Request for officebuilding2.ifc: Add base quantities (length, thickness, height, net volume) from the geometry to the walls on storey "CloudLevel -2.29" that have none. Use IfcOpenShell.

First a look at what the model holds.

```python
import ifcopenshell
import ifcopenshell.util.element
import ifcopenshell.util.unit

model = ifcopenshell.open("officebuilding2.ifc")
print(model.schema)
for unit_type in ("LENGTHUNIT", "AREAUNIT", "VOLUMEUNIT"):
    print(unit_type, ifcopenshell.util.unit.calculate_unit_scale(model, unit_type))
storey = next(s for s in model.by_type("IfcBuildingStorey") if s.Name == "CloudLevel -2.29")
walls = [e for e in ifcopenshell.util.element.get_decomposition(storey) if e.is_a("IfcWall")]
for e in sorted(walls, key=lambda e: e.id()):
    print(e.id(), e.is_a(), e.Name, list(ifcopenshell.util.element.get_psets(e, qtos_only=True)), sep=" | ")
```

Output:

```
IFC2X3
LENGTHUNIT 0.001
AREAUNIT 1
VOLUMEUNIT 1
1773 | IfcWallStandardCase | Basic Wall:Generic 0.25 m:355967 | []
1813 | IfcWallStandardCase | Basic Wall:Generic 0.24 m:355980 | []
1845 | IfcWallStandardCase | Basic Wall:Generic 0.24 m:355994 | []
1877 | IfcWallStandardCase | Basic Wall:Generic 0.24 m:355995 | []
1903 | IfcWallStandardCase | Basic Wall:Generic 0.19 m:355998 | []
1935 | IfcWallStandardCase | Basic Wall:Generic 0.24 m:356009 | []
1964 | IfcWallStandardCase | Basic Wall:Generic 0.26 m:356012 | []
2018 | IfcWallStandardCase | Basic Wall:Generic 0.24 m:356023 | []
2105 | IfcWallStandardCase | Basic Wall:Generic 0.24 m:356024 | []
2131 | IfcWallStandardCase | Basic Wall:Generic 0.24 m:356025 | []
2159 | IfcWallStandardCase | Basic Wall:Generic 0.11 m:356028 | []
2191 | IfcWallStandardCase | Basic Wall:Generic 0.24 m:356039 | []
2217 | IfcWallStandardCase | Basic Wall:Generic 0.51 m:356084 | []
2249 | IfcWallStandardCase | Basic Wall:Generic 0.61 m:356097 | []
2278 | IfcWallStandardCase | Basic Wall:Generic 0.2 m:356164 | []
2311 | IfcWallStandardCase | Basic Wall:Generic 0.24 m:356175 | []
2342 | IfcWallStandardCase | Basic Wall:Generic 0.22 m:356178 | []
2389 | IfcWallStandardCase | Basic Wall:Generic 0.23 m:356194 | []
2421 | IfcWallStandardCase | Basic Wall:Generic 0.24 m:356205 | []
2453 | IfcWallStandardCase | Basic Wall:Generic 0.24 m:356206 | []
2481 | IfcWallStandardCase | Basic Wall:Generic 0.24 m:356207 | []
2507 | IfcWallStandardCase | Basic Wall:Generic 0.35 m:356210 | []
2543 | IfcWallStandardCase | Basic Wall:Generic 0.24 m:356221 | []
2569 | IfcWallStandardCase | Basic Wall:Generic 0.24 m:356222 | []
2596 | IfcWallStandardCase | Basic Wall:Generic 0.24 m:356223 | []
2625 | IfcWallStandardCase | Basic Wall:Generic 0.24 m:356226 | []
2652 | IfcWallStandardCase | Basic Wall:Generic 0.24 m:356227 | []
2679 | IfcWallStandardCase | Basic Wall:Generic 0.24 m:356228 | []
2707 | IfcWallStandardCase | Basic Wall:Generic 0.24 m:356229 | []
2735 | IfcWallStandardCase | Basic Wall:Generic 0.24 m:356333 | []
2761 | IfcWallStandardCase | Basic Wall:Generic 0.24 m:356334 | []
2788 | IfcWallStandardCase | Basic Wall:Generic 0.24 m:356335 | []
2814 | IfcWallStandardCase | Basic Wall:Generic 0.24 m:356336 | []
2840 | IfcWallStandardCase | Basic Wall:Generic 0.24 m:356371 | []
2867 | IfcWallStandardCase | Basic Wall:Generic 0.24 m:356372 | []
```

```python
import ifcopenshell
import ifcopenshell.api.pset
import ifcopenshell.geom
import ifcopenshell.util.element
import ifcopenshell.util.shape
import ifcopenshell.util.unit

model = ifcopenshell.open("officebuilding2.ifc")
unit_scale = ifcopenshell.util.unit.calculate_unit_scale(model)
volume_scale = ifcopenshell.util.unit.calculate_unit_scale(model, "VOLUMEUNIT")
settings = ifcopenshell.geom.settings()

storey = next(s for s in model.by_type("IfcBuildingStorey") if s.Name == "CloudLevel -2.29")
walls = [e for e in ifcopenshell.util.element.get_decomposition(storey) if e.is_a("IfcWall")]

for e in sorted(walls, key=lambda e: e.id()):
    if ifcopenshell.util.element.get_psets(e, qtos_only=True, should_inherit=False):
        continue
    # Geometry comes back in metres, in the element's own axes.
    shape = ifcopenshell.geom.create_shape(settings, e)
    values = {
        "Length": ifcopenshell.util.shape.get_x(shape.geometry) / unit_scale,
        "Width": ifcopenshell.util.shape.get_y(shape.geometry) / unit_scale,
        "Height": ifcopenshell.util.shape.get_z(shape.geometry) / unit_scale,
        "NetVolume": ifcopenshell.util.shape.get_volume(shape.geometry) / volume_scale,
    }
    qto = ifcopenshell.api.pset.add_qto(model, product=e, name="BaseQuantities")
    ifcopenshell.api.pset.edit_qto(model, qto=qto, properties=values)
    print(e.id(), {k: round(v, 3) for k, v in values.items()})

model.write("officebuilding2_updated.ifc")
```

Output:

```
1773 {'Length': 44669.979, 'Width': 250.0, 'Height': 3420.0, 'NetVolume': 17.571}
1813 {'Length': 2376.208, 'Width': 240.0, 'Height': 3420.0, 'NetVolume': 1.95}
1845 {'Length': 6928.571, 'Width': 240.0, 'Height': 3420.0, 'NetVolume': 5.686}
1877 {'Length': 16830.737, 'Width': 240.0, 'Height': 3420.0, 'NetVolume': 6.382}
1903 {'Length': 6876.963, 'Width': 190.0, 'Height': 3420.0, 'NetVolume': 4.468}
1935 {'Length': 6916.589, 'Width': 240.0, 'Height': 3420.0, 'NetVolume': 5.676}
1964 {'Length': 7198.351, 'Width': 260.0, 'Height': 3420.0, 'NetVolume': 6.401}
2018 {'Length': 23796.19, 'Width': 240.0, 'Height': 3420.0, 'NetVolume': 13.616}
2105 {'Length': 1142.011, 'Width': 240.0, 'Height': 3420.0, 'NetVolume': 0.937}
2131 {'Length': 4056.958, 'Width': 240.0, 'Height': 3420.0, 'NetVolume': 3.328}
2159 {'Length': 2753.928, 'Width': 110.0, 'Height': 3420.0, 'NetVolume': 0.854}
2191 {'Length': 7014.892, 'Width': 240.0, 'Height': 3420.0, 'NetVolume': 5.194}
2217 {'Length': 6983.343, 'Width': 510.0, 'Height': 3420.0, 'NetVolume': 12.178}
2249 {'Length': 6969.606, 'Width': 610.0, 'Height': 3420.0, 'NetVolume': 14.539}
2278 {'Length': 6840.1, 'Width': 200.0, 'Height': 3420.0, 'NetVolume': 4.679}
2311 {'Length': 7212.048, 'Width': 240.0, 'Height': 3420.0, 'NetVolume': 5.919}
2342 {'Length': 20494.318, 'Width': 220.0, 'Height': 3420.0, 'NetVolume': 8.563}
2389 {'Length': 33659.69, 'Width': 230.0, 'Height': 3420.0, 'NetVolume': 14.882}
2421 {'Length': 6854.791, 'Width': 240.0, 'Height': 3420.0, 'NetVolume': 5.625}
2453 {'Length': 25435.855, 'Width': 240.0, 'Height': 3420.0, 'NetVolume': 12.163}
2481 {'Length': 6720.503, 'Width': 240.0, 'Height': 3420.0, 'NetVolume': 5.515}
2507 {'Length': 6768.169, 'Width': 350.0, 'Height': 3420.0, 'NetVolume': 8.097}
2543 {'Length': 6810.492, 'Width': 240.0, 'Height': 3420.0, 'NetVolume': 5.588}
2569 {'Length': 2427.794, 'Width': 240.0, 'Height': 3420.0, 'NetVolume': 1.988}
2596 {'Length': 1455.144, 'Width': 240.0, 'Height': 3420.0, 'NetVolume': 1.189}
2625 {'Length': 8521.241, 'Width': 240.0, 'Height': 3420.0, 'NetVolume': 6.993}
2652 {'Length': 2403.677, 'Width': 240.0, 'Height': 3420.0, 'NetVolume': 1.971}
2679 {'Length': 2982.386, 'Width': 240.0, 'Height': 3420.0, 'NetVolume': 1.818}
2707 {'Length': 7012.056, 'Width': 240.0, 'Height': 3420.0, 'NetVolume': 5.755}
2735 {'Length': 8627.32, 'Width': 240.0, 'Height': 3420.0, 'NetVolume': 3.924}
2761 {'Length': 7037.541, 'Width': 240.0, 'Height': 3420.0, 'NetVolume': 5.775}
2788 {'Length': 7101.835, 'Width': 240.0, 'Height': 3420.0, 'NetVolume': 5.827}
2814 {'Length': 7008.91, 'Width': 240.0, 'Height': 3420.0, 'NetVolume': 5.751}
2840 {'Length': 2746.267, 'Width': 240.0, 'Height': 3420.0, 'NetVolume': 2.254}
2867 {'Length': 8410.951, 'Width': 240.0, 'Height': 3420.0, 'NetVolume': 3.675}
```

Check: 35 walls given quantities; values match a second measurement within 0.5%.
